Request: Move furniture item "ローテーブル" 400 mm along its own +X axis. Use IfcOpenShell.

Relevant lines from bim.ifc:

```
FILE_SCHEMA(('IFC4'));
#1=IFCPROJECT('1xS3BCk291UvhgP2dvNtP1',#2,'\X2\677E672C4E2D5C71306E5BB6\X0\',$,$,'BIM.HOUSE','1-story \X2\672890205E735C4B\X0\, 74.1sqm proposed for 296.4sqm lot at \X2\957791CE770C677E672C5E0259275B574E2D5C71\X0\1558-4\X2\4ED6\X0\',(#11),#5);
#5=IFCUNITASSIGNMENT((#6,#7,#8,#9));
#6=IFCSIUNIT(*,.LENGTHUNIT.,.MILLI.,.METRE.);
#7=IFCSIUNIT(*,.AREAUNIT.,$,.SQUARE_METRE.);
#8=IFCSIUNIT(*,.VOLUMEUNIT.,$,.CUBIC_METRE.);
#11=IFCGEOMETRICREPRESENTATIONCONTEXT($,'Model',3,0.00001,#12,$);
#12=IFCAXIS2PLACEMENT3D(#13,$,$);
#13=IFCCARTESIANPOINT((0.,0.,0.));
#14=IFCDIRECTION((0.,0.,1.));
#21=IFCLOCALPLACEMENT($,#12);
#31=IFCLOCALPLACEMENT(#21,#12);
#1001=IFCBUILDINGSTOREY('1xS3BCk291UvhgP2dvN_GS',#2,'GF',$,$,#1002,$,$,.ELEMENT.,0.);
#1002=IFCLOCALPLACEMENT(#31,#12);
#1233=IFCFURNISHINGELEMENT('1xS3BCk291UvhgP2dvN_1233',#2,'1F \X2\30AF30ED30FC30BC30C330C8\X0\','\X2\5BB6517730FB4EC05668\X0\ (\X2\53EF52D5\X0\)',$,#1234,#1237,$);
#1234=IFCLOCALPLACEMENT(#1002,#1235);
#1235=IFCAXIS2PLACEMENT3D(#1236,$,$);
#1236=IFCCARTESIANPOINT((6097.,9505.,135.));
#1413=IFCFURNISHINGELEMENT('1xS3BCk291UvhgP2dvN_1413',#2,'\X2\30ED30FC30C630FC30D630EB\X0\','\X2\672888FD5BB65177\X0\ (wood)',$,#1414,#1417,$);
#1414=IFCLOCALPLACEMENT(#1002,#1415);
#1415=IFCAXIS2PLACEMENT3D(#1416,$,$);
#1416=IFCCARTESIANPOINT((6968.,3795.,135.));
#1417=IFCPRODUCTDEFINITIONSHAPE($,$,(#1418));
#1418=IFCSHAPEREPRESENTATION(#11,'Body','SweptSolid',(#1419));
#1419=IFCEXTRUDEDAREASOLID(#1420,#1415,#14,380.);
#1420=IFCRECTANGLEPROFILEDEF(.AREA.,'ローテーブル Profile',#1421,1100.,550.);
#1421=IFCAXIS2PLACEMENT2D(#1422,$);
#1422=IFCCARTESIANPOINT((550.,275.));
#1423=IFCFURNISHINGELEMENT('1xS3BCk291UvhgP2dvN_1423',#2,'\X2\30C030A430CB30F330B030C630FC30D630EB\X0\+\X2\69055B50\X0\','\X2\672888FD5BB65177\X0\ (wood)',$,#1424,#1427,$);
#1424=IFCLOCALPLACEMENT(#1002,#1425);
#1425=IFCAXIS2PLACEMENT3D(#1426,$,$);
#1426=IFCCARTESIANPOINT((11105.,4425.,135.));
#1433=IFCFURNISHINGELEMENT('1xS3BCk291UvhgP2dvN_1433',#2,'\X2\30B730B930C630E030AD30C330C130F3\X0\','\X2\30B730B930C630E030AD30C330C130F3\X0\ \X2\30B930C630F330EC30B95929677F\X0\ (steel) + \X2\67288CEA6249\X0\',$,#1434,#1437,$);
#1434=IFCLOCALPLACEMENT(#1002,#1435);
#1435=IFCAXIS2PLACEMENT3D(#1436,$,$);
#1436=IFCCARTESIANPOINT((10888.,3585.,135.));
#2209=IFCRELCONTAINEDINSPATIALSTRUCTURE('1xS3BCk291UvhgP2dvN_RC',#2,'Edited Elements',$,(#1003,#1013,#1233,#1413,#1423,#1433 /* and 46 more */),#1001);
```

```python
import ifcopenshell
import ifcopenshell.api.geometry
import ifcopenshell.util.placement

model = ifcopenshell.open("bim.ifc")

item = model.by_id(1413)
matrix = ifcopenshell.util.placement.get_local_placement(item.ObjectPlacement)
matrix[:3, 3] += matrix[:3, 0] * 400.0
ifcopenshell.api.geometry.edit_object_placement(model, product=item, matrix=matrix, is_si=False)

print(ifcopenshell.util.placement.get_local_placement(item.ObjectPlacement).round(3) + 0.0)

model.write("bim_v2.ifc")
```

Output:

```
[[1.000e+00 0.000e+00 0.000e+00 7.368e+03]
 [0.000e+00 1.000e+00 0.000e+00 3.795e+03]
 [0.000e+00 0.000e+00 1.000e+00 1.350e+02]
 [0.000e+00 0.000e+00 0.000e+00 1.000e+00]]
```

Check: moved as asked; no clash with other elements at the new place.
